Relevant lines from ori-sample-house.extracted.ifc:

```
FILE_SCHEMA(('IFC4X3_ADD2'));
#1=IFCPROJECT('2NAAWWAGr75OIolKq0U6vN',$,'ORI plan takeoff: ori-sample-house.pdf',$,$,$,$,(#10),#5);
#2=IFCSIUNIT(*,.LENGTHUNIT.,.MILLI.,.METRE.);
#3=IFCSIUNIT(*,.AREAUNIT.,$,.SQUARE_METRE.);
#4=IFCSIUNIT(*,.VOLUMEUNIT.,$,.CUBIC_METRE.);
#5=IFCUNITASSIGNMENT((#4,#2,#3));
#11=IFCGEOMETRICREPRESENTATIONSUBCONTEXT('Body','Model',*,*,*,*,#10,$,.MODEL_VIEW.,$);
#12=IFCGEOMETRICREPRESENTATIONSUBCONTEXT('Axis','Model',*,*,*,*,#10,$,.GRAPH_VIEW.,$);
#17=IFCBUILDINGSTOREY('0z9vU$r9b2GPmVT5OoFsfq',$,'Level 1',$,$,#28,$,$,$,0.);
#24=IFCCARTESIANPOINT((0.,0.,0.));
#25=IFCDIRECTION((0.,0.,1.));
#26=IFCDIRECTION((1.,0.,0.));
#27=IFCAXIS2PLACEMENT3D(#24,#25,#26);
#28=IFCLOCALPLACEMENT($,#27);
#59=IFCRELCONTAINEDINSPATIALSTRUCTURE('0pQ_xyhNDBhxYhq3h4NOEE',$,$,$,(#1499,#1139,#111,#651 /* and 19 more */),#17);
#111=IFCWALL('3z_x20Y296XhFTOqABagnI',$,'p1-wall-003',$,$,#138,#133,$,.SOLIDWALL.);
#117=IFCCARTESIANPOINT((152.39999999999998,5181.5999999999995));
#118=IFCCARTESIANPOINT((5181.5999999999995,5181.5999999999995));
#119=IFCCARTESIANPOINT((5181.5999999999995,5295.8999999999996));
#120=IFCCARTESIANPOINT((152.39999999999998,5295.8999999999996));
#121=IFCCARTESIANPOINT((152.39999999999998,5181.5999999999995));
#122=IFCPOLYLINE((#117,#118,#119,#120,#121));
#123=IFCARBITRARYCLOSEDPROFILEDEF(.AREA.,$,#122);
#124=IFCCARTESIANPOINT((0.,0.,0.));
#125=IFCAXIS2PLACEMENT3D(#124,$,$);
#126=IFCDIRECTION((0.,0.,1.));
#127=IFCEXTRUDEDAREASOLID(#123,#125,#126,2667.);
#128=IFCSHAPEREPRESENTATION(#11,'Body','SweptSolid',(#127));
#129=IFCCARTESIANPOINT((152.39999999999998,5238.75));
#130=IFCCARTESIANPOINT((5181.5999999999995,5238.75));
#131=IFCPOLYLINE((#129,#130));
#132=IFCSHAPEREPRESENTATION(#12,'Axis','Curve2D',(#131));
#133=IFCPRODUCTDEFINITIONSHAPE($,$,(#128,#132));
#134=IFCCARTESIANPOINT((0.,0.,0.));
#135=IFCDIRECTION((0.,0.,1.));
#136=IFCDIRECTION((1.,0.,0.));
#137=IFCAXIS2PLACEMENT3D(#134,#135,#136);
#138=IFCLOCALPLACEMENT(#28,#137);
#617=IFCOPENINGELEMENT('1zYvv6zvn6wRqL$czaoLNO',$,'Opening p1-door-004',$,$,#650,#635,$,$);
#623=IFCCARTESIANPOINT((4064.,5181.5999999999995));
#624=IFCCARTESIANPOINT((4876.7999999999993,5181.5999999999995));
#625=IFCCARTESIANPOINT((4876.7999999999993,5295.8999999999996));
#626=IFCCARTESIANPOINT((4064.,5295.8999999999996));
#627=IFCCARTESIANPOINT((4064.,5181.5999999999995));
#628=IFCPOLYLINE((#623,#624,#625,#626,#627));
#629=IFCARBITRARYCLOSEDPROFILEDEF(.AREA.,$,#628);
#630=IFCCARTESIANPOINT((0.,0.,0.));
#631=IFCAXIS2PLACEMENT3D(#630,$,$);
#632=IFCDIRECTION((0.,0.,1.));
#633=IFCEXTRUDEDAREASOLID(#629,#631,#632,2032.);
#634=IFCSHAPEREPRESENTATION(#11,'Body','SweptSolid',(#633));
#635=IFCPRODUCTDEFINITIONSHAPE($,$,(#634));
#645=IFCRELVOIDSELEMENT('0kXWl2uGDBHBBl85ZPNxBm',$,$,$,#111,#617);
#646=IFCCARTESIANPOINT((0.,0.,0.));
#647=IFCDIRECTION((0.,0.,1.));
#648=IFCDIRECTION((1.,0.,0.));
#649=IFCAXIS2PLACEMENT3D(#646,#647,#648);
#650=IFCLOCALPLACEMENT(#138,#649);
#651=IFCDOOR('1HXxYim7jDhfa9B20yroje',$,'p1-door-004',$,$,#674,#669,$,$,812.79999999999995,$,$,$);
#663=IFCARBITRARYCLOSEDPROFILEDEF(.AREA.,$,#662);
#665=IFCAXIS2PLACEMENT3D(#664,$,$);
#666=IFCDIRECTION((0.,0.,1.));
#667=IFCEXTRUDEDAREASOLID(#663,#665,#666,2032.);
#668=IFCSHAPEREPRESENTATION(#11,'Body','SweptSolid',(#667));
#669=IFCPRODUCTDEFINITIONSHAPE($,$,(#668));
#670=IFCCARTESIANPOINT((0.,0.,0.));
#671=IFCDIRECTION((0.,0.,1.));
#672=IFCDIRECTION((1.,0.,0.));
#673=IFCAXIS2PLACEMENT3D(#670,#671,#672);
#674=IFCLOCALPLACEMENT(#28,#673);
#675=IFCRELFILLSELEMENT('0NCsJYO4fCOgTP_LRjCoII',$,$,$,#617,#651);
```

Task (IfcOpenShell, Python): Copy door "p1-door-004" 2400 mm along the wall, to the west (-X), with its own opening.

```python
import ifcopenshell
import ifcopenshell.api.feature
import ifcopenshell.api.geometry
import ifcopenshell.api.root
import ifcopenshell.geom
import ifcopenshell.util.element
import ifcopenshell.util.placement
import ifcopenshell.util.shape

model = ifcopenshell.open("ori-sample-house.extracted.ifc")
settings = ifcopenshell.geom.settings()


def volume(element):
    """Net volume in cubic metres, openings subtracted."""
    shape = ifcopenshell.geom.create_shape(settings, element)
    return ifcopenshell.util.shape.get_volume(shape.geometry)


door = model.by_id(651)
opening = door.FillsVoids[0].RelatingOpeningElement
wall = opening.VoidsElements[0].RelatingBuildingElement
before = volume(wall)
shift = ifcopenshell.util.placement.get_local_placement(wall.ObjectPlacement)[:3, 0] * -2400.0

# copy_class copies the void relationship, type, container and properties, but no geometry.
new_opening = ifcopenshell.api.root.copy_class(model, product=opening)
new_opening.Representation = ifcopenshell.util.element.copy_deep(
    model, opening.Representation, exclude=["IfcGeometricRepresentationContext", "IfcRepresentationMap"]
)
new_door = ifcopenshell.api.root.copy_class(model, product=door)
new_door.Representation = ifcopenshell.util.element.copy_deep(
    model, door.Representation, exclude=["IfcGeometricRepresentationContext", "IfcRepresentationMap"]
)
ifcopenshell.api.feature.add_filling(model, opening=new_opening, element=new_door)

for old, new in ((opening, new_opening), (door, new_door)):
    matrix = ifcopenshell.util.placement.get_local_placement(old.ObjectPlacement)
    matrix[:3, 3] += shift
    ifcopenshell.api.geometry.edit_object_placement(model, product=new, matrix=matrix, is_si=False)

after = volume(wall)

print(f"wall volume {before:.3f} -> {after:.3f} m3")

model.write("ori-sample-house.extracted_rev.ifc")
```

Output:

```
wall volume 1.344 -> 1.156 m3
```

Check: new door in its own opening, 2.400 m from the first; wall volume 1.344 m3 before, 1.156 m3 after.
